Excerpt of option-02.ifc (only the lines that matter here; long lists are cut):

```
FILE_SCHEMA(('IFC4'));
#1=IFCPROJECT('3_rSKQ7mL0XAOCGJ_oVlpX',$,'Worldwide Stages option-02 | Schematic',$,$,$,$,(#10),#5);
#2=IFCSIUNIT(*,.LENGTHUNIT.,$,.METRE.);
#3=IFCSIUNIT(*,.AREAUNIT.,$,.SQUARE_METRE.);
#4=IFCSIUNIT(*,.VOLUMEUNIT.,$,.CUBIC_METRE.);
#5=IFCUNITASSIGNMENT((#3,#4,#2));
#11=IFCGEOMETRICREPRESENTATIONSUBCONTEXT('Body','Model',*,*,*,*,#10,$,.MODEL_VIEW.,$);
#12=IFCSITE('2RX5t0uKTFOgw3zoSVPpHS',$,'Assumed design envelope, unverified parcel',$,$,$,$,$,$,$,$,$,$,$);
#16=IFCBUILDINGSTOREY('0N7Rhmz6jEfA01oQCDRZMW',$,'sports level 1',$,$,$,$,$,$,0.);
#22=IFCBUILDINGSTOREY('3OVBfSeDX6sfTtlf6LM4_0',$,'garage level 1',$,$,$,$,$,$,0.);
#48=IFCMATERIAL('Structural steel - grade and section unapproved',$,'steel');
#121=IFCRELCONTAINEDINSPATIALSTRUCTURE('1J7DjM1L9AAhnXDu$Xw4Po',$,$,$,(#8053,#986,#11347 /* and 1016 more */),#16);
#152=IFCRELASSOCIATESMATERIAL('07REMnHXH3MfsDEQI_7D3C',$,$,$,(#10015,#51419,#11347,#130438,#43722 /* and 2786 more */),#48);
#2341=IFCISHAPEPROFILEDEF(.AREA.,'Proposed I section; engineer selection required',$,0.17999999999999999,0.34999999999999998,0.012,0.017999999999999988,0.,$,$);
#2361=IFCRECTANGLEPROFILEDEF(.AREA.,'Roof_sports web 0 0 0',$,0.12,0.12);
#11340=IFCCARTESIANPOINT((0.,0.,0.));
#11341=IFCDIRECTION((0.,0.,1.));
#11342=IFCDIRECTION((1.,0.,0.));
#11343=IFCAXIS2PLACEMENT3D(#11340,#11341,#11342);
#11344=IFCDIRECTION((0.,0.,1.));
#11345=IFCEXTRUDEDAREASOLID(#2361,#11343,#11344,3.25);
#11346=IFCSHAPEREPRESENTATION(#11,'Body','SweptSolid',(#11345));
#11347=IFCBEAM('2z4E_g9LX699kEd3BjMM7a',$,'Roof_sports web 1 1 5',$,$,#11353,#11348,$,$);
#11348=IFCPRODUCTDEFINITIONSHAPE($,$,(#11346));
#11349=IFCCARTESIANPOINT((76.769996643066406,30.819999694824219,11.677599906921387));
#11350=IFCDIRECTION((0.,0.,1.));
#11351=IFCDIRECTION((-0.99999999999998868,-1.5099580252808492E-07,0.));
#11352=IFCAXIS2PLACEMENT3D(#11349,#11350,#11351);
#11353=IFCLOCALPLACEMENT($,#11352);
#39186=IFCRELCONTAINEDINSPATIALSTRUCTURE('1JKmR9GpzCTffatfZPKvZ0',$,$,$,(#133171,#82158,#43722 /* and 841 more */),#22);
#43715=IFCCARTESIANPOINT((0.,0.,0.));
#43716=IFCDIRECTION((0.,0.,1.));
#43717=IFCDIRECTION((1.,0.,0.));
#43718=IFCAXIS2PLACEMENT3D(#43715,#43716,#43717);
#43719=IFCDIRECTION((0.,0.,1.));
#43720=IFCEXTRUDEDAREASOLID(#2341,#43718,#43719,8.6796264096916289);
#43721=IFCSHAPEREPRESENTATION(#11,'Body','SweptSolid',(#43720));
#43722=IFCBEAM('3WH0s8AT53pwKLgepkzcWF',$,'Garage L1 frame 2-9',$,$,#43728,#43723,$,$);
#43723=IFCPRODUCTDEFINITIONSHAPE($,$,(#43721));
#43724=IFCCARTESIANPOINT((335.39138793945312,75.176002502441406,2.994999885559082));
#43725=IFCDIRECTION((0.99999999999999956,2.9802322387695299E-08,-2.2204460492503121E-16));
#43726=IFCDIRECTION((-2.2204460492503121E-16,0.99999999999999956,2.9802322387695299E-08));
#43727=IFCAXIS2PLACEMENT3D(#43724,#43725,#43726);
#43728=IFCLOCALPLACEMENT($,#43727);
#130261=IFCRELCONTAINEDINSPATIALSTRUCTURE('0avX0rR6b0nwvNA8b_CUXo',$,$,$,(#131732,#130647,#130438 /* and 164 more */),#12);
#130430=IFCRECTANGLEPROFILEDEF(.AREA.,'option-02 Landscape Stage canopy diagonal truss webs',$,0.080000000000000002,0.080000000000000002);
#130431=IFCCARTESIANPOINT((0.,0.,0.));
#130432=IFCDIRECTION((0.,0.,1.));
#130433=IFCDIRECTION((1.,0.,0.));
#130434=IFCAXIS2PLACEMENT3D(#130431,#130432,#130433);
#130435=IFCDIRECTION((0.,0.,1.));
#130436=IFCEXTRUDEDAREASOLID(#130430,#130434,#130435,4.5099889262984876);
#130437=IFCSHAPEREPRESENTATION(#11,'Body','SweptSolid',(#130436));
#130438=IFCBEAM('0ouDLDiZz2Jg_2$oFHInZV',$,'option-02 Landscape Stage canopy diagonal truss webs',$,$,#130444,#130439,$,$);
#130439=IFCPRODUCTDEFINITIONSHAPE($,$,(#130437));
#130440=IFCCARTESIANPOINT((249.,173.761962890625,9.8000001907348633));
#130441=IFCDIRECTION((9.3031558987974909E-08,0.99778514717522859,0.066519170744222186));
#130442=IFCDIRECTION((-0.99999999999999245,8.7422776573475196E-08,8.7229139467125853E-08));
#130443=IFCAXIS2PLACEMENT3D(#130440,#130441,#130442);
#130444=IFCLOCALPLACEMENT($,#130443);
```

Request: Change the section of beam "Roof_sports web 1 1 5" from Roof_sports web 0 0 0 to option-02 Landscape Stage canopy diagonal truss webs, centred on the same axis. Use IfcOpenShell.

```python
import ifcopenshell
import ifcopenshell.util.element
import ifcopenshell.util.representation

model = ifcopenshell.open("option-02.ifc")

member = model.by_id(11347)
source = next(p for p in model.by_type("IfcRectangleProfileDef") if p.ProfileName == "option-02 Landscape Stage canopy diagonal truss webs")

body = ifcopenshell.util.representation.get_representation(member, "Model", "Body")
solid = body.Items[0]
old_profile = solid.SweptArea

# Copy the section's sizes but keep this member's own profile position.
profile = ifcopenshell.util.element.copy(model, source)
profile.Position = old_profile.Position
solid.SweptArea = profile
if not model.get_total_inverses(old_profile):
    ifcopenshell.util.element.remove_deep2(model, old_profile)

print(solid.SweptArea)

model.write("option-02_updated.ifc")
```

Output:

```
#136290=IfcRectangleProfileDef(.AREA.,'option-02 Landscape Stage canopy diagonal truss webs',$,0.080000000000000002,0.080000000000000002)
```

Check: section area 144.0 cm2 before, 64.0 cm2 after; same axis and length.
